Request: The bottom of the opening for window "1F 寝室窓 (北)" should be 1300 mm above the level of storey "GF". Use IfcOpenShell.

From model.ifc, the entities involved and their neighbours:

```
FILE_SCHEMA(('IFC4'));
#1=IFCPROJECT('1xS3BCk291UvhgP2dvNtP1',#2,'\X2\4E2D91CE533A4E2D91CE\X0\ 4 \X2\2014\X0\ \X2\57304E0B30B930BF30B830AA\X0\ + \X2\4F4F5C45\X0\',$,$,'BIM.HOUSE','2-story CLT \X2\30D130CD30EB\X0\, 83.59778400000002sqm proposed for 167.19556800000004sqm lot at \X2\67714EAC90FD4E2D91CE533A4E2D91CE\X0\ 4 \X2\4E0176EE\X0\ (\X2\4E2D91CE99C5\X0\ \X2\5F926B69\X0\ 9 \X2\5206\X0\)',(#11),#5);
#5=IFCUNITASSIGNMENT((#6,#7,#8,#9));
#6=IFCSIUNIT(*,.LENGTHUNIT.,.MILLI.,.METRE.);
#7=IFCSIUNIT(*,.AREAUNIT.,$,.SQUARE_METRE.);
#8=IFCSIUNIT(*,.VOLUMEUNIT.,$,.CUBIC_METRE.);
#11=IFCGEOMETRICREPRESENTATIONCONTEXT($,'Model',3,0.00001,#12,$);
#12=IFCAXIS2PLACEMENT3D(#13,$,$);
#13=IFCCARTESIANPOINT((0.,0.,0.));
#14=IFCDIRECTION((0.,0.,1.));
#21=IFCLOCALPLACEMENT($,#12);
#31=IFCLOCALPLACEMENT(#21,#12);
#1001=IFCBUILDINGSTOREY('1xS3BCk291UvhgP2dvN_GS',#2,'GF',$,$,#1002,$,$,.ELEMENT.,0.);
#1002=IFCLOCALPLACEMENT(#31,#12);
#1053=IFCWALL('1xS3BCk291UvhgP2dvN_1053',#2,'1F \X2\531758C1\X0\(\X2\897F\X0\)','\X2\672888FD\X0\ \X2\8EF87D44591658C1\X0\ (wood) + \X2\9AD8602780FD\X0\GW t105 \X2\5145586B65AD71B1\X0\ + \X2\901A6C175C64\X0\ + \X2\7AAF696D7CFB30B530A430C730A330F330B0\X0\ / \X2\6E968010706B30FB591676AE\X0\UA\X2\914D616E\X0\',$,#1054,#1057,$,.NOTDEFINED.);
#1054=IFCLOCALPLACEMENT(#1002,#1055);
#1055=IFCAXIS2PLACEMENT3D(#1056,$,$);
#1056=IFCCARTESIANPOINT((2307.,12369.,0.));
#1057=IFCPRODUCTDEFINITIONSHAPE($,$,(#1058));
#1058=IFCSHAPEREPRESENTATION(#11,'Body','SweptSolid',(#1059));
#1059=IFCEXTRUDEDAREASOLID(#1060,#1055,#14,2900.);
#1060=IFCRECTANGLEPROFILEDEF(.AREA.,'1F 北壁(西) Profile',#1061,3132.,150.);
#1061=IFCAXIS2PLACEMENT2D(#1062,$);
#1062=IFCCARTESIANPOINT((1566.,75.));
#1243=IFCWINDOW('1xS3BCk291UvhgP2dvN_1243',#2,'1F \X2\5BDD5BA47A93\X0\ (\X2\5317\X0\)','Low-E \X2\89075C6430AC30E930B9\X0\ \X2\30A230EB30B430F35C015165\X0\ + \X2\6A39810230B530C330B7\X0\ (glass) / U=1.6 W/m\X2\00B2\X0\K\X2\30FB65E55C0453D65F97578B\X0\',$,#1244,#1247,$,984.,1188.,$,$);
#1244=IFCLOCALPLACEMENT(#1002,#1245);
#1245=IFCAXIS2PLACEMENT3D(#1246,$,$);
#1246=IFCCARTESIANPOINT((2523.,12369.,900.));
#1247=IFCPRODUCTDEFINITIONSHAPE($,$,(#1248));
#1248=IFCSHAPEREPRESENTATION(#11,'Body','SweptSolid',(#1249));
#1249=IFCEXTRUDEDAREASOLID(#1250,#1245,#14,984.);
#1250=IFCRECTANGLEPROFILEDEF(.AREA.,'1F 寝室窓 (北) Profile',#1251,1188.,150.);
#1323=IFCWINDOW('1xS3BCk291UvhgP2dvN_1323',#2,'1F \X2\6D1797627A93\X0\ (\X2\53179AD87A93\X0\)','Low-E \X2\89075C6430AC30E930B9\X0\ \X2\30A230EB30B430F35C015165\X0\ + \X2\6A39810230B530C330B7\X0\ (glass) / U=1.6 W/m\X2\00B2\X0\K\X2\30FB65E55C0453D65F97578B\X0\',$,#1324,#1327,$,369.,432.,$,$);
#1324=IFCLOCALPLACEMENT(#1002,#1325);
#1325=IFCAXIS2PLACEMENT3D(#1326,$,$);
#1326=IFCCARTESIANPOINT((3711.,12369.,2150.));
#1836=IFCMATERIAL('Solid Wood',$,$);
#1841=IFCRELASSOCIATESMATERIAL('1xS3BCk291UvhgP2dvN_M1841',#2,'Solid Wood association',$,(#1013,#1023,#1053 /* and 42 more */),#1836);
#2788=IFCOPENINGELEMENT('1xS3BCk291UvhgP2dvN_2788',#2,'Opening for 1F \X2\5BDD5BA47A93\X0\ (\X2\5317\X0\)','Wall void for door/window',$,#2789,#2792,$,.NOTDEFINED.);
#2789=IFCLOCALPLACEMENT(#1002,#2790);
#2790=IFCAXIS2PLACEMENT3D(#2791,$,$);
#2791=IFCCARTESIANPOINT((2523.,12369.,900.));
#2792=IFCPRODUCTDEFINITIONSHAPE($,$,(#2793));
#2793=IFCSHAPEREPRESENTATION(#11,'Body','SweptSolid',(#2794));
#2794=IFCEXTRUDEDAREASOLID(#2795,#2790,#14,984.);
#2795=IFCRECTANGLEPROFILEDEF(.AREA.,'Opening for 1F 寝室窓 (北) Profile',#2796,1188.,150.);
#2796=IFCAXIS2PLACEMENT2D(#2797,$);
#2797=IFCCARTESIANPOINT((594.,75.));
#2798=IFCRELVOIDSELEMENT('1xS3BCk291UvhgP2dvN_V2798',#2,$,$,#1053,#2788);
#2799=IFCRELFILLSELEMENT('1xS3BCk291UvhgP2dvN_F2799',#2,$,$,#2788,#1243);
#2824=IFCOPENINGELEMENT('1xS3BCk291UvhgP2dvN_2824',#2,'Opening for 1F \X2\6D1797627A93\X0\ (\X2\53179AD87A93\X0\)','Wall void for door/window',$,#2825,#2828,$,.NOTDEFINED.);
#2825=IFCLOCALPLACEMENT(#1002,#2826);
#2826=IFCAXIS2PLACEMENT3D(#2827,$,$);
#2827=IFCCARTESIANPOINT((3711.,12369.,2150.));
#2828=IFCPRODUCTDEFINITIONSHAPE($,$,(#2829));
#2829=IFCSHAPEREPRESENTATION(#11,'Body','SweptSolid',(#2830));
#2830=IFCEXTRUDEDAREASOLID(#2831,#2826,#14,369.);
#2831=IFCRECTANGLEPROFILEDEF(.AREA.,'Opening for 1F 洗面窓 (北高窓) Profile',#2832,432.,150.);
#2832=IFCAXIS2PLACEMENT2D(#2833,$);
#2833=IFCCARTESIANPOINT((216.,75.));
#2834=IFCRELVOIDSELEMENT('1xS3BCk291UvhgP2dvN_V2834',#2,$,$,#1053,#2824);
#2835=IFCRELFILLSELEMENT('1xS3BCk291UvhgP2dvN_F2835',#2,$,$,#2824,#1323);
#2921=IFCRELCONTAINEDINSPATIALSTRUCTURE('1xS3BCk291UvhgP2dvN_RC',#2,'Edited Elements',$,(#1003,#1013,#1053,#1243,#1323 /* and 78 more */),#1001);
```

```python
import numpy as np
import ifcopenshell
import ifcopenshell.api.geometry
import ifcopenshell.geom
import ifcopenshell.util.element
import ifcopenshell.util.placement
import ifcopenshell.util.shape
import ifcopenshell.util.unit

model = ifcopenshell.open("model.ifc")
unit_scale = ifcopenshell.util.unit.calculate_unit_scale(model)

window = model.by_guid("1xS3BCk291UvhgP2dvN_1243")
opening = window.FillsVoids[0].RelatingOpeningElement
storey = ifcopenshell.util.element.get_container(window, ifc_class="IfcBuildingStorey")
level = ifcopenshell.util.placement.get_local_placement(storey.ObjectPlacement)[2, 3]

# The opening's origin need not be at the sill, so measure its lowest point.
shape = ifcopenshell.geom.create_shape(ifcopenshell.geom.settings(), opening)
bottom = ifcopenshell.util.shape.get_shape_bottom_elevation(shape, shape.geometry) / unit_scale
dz = level + 1300.0 - bottom

shift = np.array([0.0, 0.0, dz])
# The window is not placed relative to its opening, so move both.
for product in (opening, window):
    matrix = ifcopenshell.util.placement.get_local_placement(product.ObjectPlacement)
    matrix[:3, 3] += shift
    ifcopenshell.api.geometry.edit_object_placement(model, product=product, matrix=matrix, is_si=False)

print(f"moved by {dz * unit_scale:+.3f} m")

model.write("model_v2.ifc")
```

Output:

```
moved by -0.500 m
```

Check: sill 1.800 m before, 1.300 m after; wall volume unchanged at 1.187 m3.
